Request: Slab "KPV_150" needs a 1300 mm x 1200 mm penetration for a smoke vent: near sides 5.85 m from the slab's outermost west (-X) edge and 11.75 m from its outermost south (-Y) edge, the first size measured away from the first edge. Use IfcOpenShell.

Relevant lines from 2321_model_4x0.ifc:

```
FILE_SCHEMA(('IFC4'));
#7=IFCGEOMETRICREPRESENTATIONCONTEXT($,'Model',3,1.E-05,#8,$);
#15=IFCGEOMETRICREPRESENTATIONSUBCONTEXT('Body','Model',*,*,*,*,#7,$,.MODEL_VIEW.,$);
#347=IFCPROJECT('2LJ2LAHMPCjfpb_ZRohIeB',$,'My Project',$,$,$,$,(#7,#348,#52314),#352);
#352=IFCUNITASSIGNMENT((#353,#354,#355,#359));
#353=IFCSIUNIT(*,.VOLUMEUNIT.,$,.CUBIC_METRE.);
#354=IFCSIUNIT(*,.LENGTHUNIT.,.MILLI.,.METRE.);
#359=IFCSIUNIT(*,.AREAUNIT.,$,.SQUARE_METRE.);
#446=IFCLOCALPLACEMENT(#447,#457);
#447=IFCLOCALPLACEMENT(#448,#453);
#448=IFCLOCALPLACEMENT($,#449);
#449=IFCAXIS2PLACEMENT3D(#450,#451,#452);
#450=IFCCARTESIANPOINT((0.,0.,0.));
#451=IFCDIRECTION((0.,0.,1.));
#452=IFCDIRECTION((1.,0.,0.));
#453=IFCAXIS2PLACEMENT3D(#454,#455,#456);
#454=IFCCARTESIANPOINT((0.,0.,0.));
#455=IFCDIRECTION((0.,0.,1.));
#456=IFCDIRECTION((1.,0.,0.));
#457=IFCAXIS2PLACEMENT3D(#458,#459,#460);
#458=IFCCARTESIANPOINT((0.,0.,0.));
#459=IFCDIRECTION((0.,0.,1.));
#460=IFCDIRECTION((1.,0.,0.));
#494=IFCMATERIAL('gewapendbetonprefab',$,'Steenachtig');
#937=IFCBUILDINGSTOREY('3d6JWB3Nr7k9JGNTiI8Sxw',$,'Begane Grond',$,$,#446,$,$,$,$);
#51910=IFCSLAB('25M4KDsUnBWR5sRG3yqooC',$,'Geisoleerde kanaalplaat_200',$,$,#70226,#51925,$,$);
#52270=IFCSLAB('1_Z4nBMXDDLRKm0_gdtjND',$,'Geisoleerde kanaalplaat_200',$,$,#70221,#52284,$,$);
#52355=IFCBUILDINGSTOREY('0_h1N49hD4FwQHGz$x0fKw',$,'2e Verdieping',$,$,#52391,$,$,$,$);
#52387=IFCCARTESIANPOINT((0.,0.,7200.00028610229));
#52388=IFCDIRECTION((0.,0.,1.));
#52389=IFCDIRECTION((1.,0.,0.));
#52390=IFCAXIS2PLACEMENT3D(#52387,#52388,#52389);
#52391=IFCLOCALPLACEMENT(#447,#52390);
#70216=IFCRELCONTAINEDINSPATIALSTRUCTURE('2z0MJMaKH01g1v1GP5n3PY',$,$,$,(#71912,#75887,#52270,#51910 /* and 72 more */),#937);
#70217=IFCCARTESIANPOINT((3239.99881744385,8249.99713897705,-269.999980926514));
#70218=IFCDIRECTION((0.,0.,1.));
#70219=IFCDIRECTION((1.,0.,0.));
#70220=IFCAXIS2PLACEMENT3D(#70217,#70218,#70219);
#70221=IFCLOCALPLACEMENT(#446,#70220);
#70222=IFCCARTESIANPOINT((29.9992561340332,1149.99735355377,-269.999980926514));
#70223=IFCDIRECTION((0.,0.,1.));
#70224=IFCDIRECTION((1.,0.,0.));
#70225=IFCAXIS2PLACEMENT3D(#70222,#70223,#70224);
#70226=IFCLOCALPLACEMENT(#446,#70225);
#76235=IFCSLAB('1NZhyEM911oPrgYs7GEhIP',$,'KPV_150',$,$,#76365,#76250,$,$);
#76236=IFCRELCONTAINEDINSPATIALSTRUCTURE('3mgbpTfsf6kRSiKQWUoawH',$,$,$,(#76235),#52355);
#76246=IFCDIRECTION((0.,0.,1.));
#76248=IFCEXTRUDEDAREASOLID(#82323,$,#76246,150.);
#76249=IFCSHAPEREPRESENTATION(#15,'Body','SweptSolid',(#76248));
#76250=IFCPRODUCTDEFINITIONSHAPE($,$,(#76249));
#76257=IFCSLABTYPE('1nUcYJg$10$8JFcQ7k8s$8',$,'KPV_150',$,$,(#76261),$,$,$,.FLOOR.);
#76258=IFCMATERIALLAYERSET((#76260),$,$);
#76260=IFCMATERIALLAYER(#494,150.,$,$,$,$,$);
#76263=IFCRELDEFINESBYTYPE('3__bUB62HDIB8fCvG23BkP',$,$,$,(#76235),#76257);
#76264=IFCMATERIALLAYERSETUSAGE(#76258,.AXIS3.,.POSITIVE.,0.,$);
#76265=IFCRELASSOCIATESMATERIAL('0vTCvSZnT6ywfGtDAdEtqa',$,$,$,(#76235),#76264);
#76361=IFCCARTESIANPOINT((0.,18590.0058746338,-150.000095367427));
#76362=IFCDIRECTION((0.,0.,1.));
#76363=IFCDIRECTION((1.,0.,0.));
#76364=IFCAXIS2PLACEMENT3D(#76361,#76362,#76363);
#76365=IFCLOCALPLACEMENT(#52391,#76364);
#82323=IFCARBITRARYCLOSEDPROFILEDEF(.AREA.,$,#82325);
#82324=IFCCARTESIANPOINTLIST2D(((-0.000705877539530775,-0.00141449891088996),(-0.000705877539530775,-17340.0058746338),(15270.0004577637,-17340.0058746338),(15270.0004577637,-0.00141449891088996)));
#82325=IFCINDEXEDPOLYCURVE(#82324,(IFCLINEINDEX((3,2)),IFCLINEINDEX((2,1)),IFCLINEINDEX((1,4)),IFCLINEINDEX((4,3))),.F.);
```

```python
import numpy as np
import ifcopenshell
import ifcopenshell.api.feature
import ifcopenshell.api.geometry
import ifcopenshell.api.root
import ifcopenshell.geom
import ifcopenshell.util.placement
import ifcopenshell.util.representation
import ifcopenshell.util.shape
import ifcopenshell.util.unit

model = ifcopenshell.open("2321_model_4x0.ifc")
unit_scale = ifcopenshell.util.unit.calculate_unit_scale(model)
settings = ifcopenshell.geom.settings()


def volume(element):
    """Net volume in cubic metres, openings subtracted."""
    shape = ifcopenshell.geom.create_shape(settings, element)
    return ifcopenshell.util.shape.get_volume(shape.geometry)


slab = model.by_guid("1NZhyEM911oPrgYs7GEhIP")
before = volume(slab)

# Extent in the slab's own axes, in metres. The edges named are its -X and -Y sides.
slab_shape = ifcopenshell.geom.create_shape(settings, slab)
vertices = ifcopenshell.util.shape.get_vertices(slab_shape.geometry)
x_min, y_min, bottom = vertices.min(axis=0)
top = vertices[:, 2].max()

opening = ifcopenshell.api.root.create_entity(model, ifc_class="IfcOpeningElement", name="Smoke vent opening", predefined_type="OPENING")
context = ifcopenshell.util.representation.get_context(model, "Model", "Body", "MODEL_VIEW")
width, depth = 1.3, 1.2
outline = [(0.0, 0.0), (width, 0.0), (width, depth), (0.0, depth), (0.0, 0.0)]
# Overshoot both faces by 50 mm so the cut is clean.
shape = ifcopenshell.api.geometry.add_slab_representation(
    model, context=context, depth=top - bottom + 0.1, polyline=outline
)
ifcopenshell.api.geometry.assign_representation(model, product=opening, representation=shape)

matrix = ifcopenshell.util.placement.get_local_placement(slab.ObjectPlacement)
matrix[:, 3] = matrix @ np.append(np.array([x_min + 5.85, y_min + 11.75, bottom - 0.05]) / unit_scale, 1.0)
ifcopenshell.api.geometry.edit_object_placement(model, product=opening, matrix=matrix, is_si=False)
ifcopenshell.api.feature.add_feature(model, feature=opening, element=slab)

after = volume(slab)

print(f"slab volume {before:.3f} -> {after:.3f} m3")

model.write("2321_model_4x0_edited.ifc")
```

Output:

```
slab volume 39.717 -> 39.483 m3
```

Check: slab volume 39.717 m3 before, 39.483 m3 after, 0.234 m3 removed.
